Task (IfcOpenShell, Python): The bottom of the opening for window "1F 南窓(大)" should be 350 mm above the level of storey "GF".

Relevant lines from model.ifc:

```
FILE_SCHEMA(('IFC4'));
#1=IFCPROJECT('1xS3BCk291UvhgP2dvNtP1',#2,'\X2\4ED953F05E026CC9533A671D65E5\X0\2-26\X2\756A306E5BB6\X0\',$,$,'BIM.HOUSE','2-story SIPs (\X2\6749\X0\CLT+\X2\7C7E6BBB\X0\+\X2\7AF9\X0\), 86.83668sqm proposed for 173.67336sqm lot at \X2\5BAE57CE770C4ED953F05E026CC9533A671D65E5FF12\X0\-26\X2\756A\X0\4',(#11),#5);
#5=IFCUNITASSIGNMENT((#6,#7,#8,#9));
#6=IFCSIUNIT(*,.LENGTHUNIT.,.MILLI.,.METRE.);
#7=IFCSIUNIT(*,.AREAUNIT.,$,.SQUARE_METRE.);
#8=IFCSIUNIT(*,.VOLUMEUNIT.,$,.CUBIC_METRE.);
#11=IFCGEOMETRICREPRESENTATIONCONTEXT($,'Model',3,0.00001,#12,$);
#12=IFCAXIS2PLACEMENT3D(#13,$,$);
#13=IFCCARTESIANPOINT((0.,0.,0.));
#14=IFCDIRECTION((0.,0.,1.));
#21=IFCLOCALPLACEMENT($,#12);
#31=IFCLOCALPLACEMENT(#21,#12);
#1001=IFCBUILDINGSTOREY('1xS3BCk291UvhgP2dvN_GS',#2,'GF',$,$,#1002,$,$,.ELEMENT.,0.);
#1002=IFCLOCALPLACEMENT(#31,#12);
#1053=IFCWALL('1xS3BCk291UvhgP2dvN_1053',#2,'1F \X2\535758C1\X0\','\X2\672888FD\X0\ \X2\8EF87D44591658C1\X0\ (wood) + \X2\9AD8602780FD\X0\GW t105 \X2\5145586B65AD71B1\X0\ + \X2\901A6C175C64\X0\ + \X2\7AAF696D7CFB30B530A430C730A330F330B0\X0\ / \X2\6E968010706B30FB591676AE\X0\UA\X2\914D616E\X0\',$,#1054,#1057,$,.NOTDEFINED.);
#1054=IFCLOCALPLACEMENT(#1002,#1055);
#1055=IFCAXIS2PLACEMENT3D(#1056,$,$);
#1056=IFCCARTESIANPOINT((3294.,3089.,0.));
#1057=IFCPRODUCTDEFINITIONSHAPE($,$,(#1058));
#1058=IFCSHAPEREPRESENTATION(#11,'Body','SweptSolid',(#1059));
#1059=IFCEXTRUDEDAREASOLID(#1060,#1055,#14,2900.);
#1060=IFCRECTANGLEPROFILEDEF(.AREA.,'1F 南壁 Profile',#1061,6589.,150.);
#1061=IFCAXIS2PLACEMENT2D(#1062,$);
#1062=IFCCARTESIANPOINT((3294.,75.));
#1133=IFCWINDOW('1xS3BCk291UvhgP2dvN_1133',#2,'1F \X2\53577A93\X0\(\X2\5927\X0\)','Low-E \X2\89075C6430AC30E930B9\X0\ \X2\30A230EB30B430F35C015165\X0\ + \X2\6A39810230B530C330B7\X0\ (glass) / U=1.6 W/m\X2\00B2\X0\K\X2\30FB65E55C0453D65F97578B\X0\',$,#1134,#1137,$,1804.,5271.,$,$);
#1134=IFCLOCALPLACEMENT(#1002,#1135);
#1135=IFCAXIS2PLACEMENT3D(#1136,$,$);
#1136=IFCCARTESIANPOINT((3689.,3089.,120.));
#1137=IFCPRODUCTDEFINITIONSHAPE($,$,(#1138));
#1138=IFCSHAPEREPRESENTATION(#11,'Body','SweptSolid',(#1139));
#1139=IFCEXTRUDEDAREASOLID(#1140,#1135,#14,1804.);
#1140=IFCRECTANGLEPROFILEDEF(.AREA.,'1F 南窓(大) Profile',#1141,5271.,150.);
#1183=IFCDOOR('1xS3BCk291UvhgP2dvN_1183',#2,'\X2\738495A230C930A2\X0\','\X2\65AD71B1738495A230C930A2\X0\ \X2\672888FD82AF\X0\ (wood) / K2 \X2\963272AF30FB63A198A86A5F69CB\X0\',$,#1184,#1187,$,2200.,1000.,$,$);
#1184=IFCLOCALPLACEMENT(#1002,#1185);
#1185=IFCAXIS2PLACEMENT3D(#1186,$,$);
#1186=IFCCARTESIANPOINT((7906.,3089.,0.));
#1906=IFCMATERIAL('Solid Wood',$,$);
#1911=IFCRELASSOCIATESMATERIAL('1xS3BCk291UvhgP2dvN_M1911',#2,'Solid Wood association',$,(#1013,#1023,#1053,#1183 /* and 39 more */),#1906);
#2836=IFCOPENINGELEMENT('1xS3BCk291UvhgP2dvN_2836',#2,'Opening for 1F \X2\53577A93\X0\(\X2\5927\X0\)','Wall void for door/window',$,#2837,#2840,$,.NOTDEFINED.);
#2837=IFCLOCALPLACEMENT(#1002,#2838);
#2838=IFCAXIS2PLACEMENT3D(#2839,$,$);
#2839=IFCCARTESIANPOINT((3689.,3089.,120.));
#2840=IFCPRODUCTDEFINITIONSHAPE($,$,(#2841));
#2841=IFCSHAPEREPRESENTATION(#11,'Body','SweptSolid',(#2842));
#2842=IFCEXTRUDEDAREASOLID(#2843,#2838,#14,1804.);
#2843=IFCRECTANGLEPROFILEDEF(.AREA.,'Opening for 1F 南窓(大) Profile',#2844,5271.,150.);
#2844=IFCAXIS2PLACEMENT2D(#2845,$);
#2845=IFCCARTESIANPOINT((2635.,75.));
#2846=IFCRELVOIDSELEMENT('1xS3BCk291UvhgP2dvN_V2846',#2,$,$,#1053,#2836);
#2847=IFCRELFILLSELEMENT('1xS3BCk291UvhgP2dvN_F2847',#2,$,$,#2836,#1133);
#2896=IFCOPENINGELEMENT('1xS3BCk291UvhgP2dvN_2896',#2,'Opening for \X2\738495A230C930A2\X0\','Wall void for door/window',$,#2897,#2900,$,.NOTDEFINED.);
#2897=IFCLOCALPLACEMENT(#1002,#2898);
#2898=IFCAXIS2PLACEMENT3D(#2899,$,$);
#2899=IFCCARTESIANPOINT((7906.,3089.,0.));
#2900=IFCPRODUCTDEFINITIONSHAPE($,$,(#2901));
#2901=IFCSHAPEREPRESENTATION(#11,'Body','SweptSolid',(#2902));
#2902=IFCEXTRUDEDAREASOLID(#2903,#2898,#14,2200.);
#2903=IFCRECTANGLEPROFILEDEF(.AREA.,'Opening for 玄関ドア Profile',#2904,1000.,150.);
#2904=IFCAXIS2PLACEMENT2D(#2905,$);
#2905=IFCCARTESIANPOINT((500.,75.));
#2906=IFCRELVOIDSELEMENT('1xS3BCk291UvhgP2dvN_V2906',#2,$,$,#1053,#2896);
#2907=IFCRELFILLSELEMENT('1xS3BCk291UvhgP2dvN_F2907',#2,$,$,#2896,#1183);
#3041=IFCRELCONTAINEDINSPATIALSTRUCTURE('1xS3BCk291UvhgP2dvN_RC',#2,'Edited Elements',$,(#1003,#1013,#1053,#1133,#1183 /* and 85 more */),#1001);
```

```python
import numpy as np
import ifcopenshell
import ifcopenshell.api.geometry
import ifcopenshell.geom
import ifcopenshell.util.element
import ifcopenshell.util.placement
import ifcopenshell.util.shape
import ifcopenshell.util.unit

model = ifcopenshell.open("model.ifc")
unit_scale = ifcopenshell.util.unit.calculate_unit_scale(model)

window = model.by_guid("1xS3BCk291UvhgP2dvN_1133")
opening = window.FillsVoids[0].RelatingOpeningElement
storey = ifcopenshell.util.element.get_container(window, ifc_class="IfcBuildingStorey")
level = ifcopenshell.util.placement.get_local_placement(storey.ObjectPlacement)[2, 3]

# The opening's origin need not be at the sill, so measure its lowest point.
shape = ifcopenshell.geom.create_shape(ifcopenshell.geom.settings(), opening)
bottom = ifcopenshell.util.shape.get_shape_bottom_elevation(shape, shape.geometry) / unit_scale
dz = level + 0.35 / unit_scale - bottom

shift = np.array([0.0, 0.0, dz])
# The window is not placed relative to its opening, so move both.
for product in (opening, window):
    matrix = ifcopenshell.util.placement.get_local_placement(product.ObjectPlacement)
    matrix[:3, 3] += shift
    ifcopenshell.api.geometry.edit_object_placement(model, product=product, matrix=matrix, is_si=False)

print(f"moved by {dz * unit_scale:+.3f} m")

model.write("model_updated.ifc")
```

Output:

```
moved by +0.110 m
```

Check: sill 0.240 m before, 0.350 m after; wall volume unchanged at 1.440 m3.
